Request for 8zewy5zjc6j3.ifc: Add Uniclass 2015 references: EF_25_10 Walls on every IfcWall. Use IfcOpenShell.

First a look at what the model holds.

```python
import ifcopenshell

model = ifcopenshell.open("8zewy5zjc6j3.ifc")
print(model.schema)
print("classifications:", [c.Name for c in model.by_type("IfcClassification")])
for ifc_class in ("IfcDoor", "IfcRoof", "IfcStair", "IfcWall", "IfcWindow"):
    print(ifc_class, len(model.by_type(ifc_class)))
```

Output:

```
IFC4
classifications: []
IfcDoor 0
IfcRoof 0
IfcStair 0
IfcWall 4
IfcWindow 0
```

```python
import ifcopenshell
import ifcopenshell.api.classification

model = ifcopenshell.open("8zewy5zjc6j3.ifc")

system = ifcopenshell.api.classification.add_classification(model, classification="Uniclass 2015")

codes = {
    "IfcWall": ("EF_25_10", "Walls"),
}
for ifc_class, (code, name) in codes.items():
    products = model.by_type(ifc_class)
    ifcopenshell.api.classification.add_reference(
        model, products=products, classification=system, identification=code, name=name
    )
    print(code, len(products))

model.write("8zewy5zjc6j3_updated.ifc")
```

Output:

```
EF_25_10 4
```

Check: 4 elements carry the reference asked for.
